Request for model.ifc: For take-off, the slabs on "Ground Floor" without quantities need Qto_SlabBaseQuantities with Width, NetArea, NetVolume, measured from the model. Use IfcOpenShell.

First a look at what the model holds.

```python
import ifcopenshell
import ifcopenshell.util.element
import ifcopenshell.util.unit

model = ifcopenshell.open("model.ifc")
print(model.schema)
for unit_type in ("LENGTHUNIT", "AREAUNIT", "VOLUMEUNIT"):
    print(unit_type, ifcopenshell.util.unit.calculate_unit_scale(model, unit_type))
storey = next(s for s in model.by_type("IfcBuildingStorey") if s.Name == "Ground Floor")
slabs = [e for e in ifcopenshell.util.element.get_decomposition(storey) if e.is_a("IfcSlab")]
for e in sorted(slabs, key=lambda e: e.id()):
    print(e.id(), e.is_a(), e.Name, list(ifcopenshell.util.element.get_psets(e, qtos_only=True)), sep=" | ")
```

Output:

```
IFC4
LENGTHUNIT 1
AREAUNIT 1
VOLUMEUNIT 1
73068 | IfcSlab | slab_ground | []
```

```python
import ifcopenshell
import ifcopenshell.api.pset
import ifcopenshell.geom
import ifcopenshell.util.element
import ifcopenshell.util.shape
import ifcopenshell.util.unit

model = ifcopenshell.open("model.ifc")
unit_scale = ifcopenshell.util.unit.calculate_unit_scale(model)
area_scale = ifcopenshell.util.unit.calculate_unit_scale(model, "AREAUNIT")
volume_scale = ifcopenshell.util.unit.calculate_unit_scale(model, "VOLUMEUNIT")
settings = ifcopenshell.geom.settings()

storey = next(s for s in model.by_type("IfcBuildingStorey") if s.Name == "Ground Floor")
slabs = [e for e in ifcopenshell.util.element.get_decomposition(storey) if e.is_a("IfcSlab")]

for e in sorted(slabs, key=lambda e: e.id()):
    if ifcopenshell.util.element.get_psets(e, qtos_only=True, should_inherit=False):
        continue
    # Geometry comes back in metres, in the element's own axes.
    shape = ifcopenshell.geom.create_shape(settings, e)
    values = {
        "Width": ifcopenshell.util.shape.get_z(shape.geometry) / unit_scale,
        "NetArea": ifcopenshell.util.shape.get_footprint_area(shape.geometry) / area_scale,
        "NetVolume": ifcopenshell.util.shape.get_volume(shape.geometry) / volume_scale,
    }
    qto = ifcopenshell.api.pset.add_qto(model, product=e, name="Qto_SlabBaseQuantities")
    ifcopenshell.api.pset.edit_qto(model, qto=qto, properties=values)
    print(e.id(), {k: round(v, 3) for k, v in values.items()})

model.write("model_v2.ifc")
```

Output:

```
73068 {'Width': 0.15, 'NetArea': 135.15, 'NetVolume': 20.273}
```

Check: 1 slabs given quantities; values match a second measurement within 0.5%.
